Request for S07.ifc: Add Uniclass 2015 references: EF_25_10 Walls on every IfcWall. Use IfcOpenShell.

First a look at what the model holds.

```python
import ifcopenshell

model = ifcopenshell.open("S07.ifc")
print(model.schema)
print("classifications:", [c.Name for c in model.by_type("IfcClassification")])
for ifc_class in ("IfcDoor", "IfcRoof", "IfcStair", "IfcWall", "IfcWindow"):
    print(ifc_class, len(model.by_type(ifc_class)))
```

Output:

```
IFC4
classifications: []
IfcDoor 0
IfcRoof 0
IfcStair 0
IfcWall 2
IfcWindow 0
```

```python
import ifcopenshell
import ifcopenshell.api.classification

model = ifcopenshell.open("S07.ifc")

system = ifcopenshell.api.classification.add_classification(model, classification="Uniclass 2015")

codes = {
    "IfcWall": ("EF_25_10", "Walls"),
}
for ifc_class, (code, name) in codes.items():
    products = model.by_type(ifc_class)
    ifcopenshell.api.classification.add_reference(
        model, products=products, classification=system, identification=code, name=name
    )
    print(code, len(products))

model.write("S07_edited.ifc")
```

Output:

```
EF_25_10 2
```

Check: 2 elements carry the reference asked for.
